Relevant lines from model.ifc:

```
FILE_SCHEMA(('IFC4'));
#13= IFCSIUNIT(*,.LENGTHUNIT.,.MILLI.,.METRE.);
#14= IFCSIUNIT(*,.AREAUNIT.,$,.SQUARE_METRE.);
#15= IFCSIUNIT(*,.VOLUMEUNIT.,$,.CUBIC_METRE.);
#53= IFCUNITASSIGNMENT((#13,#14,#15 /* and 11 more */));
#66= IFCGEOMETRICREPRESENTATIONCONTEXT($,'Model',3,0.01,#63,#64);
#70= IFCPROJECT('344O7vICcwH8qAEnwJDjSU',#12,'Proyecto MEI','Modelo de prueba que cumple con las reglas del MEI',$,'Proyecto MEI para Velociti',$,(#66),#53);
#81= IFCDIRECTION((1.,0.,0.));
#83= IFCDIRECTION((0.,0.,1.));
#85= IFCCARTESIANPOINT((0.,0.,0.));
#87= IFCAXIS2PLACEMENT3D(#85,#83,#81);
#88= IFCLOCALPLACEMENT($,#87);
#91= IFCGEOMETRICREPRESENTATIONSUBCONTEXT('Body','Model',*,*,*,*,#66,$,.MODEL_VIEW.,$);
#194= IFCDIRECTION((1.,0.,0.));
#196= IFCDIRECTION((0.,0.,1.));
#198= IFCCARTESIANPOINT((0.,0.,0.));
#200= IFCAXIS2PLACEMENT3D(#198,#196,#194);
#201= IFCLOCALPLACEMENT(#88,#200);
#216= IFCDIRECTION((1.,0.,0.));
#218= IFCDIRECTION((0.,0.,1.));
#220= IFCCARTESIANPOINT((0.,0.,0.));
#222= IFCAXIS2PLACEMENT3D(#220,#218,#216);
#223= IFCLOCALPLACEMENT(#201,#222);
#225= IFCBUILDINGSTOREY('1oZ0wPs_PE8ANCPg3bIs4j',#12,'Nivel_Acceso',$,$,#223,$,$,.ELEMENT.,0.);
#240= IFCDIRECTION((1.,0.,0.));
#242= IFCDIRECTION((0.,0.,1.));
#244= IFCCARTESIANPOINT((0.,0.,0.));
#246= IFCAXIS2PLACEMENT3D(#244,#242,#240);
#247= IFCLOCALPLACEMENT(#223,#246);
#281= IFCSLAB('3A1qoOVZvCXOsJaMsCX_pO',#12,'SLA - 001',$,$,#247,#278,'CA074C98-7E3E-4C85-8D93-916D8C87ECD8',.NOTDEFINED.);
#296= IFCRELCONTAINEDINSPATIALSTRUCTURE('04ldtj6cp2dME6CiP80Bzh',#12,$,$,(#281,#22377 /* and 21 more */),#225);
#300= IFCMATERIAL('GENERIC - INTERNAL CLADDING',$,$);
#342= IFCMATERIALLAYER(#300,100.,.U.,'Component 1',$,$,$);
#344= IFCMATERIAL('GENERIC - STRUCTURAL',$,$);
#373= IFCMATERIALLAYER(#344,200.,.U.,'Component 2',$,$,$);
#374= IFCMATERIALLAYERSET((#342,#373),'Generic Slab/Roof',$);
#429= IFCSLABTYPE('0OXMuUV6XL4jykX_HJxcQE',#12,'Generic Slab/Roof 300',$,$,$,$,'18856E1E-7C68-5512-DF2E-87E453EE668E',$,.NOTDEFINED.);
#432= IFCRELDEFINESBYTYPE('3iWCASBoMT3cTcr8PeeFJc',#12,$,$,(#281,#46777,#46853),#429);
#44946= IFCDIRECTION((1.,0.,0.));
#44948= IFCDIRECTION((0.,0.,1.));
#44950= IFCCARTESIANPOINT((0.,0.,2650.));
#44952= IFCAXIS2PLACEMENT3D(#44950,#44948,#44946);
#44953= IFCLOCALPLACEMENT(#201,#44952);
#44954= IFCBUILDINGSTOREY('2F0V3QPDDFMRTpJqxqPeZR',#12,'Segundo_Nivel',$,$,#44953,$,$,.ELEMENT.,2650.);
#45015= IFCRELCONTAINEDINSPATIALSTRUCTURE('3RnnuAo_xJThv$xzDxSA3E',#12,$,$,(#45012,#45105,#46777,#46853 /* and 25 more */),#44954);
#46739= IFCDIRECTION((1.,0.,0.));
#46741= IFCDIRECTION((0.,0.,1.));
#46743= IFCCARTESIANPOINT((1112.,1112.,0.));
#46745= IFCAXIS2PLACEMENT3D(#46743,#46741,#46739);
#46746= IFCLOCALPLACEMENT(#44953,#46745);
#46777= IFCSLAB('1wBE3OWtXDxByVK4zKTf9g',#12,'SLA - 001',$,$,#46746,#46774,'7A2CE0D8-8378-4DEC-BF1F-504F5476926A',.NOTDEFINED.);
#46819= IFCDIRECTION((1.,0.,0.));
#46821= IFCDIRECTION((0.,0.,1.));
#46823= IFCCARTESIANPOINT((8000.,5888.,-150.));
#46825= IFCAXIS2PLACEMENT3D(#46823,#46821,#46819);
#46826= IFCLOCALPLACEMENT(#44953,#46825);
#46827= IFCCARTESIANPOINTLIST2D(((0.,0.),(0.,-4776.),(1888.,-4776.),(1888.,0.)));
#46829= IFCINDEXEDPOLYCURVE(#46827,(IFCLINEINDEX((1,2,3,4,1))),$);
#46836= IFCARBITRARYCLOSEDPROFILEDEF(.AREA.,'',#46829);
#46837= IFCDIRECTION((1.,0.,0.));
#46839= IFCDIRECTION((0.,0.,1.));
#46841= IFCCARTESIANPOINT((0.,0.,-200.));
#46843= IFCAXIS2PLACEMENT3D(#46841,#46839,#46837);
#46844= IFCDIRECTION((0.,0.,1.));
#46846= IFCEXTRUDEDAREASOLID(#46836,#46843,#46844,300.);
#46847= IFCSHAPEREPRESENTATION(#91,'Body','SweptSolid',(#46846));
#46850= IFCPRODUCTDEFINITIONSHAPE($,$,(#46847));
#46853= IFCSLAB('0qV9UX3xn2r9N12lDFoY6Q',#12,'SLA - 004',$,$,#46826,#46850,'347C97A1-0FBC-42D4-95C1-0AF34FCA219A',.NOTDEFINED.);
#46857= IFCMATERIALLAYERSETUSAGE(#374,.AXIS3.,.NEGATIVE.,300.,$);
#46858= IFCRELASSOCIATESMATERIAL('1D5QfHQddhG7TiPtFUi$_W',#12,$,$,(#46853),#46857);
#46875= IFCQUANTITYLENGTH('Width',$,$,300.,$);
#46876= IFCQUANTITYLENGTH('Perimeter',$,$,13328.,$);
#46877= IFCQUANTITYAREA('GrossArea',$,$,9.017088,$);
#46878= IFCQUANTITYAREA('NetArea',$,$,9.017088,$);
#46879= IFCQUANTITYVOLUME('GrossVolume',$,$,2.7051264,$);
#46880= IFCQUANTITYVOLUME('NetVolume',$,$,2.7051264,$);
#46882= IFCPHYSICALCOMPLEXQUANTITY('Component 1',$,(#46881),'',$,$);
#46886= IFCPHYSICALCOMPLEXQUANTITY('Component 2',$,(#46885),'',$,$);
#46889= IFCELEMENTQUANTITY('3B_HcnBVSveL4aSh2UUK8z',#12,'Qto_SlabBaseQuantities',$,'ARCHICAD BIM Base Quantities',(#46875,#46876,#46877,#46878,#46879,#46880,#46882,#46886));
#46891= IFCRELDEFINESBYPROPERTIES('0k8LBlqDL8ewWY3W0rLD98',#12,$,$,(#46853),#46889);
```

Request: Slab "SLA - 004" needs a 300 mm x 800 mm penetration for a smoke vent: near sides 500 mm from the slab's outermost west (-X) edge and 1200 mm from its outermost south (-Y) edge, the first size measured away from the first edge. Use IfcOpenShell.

```python
import numpy as np
import ifcopenshell
import ifcopenshell.api.feature
import ifcopenshell.api.geometry
import ifcopenshell.api.pset
import ifcopenshell.api.root
import ifcopenshell.geom
import ifcopenshell.util.element
import ifcopenshell.util.placement
import ifcopenshell.util.representation
import ifcopenshell.util.shape
import ifcopenshell.util.unit

model = ifcopenshell.open("model.ifc")
unit_scale = ifcopenshell.util.unit.calculate_unit_scale(model)
area_scale = ifcopenshell.util.unit.calculate_unit_scale(model, "AREAUNIT")
volume_scale = ifcopenshell.util.unit.calculate_unit_scale(model, "VOLUMEUNIT")
settings = ifcopenshell.geom.settings()


def volume(element):
    """Net volume in cubic metres, openings subtracted."""
    shape = ifcopenshell.geom.create_shape(settings, element)
    return ifcopenshell.util.shape.get_volume(shape.geometry)


slab = model.by_guid("0qV9UX3xn2r9N12lDFoY6Q")
before = volume(slab)

# Extent in the slab's own axes, in metres. The edges named are its -X and -Y sides.
slab_shape = ifcopenshell.geom.create_shape(settings, slab)
vertices = ifcopenshell.util.shape.get_vertices(slab_shape.geometry)
x_min, y_min, bottom = vertices.min(axis=0)
top = vertices[:, 2].max()

opening = ifcopenshell.api.root.create_entity(model, ifc_class="IfcOpeningElement", name="Smoke vent opening", predefined_type="OPENING")
context = ifcopenshell.util.representation.get_context(model, "Model", "Body", "MODEL_VIEW")
width, depth = 0.3, 0.8
outline = [(0.0, 0.0), (width, 0.0), (width, depth), (0.0, depth), (0.0, 0.0)]
# Overshoot both faces by 50 mm so the cut is clean.
shape = ifcopenshell.api.geometry.add_slab_representation(
    model, context=context, depth=top - bottom + 0.1, polyline=outline
)
ifcopenshell.api.geometry.assign_representation(model, product=opening, representation=shape)

matrix = ifcopenshell.util.placement.get_local_placement(slab.ObjectPlacement)
matrix[:, 3] = matrix @ np.append(np.array([x_min + 0.5, y_min + 1.2, bottom - 0.05]) / unit_scale, 1.0)
ifcopenshell.api.geometry.edit_object_placement(model, product=opening, matrix=matrix, is_si=False)
ifcopenshell.api.feature.add_feature(model, feature=opening, element=slab)

after = volume(slab)

# Update the slab's stored quantities.
qto = model.by_id(ifcopenshell.util.element.get_pset(slab, "Qto_SlabBaseQuantities", should_inherit=False)["id"])
ifcopenshell.api.pset.edit_qto(model, qto=qto, properties={
    "NetArea": after / (top - bottom) / area_scale,
    "NetVolume": after / volume_scale,
})

print(f"slab volume {before:.3f} -> {after:.3f} m3")

model.write("model_v2.ifc")
```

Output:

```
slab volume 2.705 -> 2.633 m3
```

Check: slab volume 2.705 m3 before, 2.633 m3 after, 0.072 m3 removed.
